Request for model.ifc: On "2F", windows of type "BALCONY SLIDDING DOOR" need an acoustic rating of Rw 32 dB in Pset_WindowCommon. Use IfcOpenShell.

First a look at what the model holds.

```python
import ifcopenshell
import ifcopenshell.util.element

model = ifcopenshell.open("model.ifc")
print(model.schema)
storey = next(s for s in model.by_type("IfcBuildingStorey") if s.Name == "2F")
windows = [e for e in ifcopenshell.util.element.get_decomposition(storey) if e.is_a("IfcWindow")]
seen = {}
for e in windows:
    element_type = ifcopenshell.util.element.get_type(e)
    key = (element_type.Name if element_type != e and element_type else None, ifcopenshell.util.element.get_pset(e, "Pset_WindowCommon", "AcousticRating"))
    seen[key] = seen.get(key, 0) + 1
for (name, value), count in sorted(seen.items(), key=str):
    print(count, "x", name, "|", value)
```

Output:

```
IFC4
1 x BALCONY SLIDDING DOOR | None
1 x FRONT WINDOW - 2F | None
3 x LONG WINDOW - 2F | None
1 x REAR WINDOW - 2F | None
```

```python
import ifcopenshell
import ifcopenshell.api.pset
import ifcopenshell.util.element

model = ifcopenshell.open("model.ifc")

storey = next(s for s in model.by_type("IfcBuildingStorey") if s.Name == "2F")
windows = [e for e in ifcopenshell.util.element.get_decomposition(storey) if e.is_a("IfcWindow")]

count = 0
for e in windows:
    element_type = ifcopenshell.util.element.get_type(e)
    if element_type in (None, e) or element_type.Name != "BALCONY SLIDDING DOOR":
        continue
    # add_pset returns the element's existing set when there is one.
    pset = ifcopenshell.api.pset.add_pset(model, product=e, name="Pset_WindowCommon")
    ifcopenshell.api.pset.edit_pset(model, pset=pset, properties={"AcousticRating": "Rw 32 dB"})
    count += 1

print(count, "windows updated")

model.write("model_edited.ifc")
```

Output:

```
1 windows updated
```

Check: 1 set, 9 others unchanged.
